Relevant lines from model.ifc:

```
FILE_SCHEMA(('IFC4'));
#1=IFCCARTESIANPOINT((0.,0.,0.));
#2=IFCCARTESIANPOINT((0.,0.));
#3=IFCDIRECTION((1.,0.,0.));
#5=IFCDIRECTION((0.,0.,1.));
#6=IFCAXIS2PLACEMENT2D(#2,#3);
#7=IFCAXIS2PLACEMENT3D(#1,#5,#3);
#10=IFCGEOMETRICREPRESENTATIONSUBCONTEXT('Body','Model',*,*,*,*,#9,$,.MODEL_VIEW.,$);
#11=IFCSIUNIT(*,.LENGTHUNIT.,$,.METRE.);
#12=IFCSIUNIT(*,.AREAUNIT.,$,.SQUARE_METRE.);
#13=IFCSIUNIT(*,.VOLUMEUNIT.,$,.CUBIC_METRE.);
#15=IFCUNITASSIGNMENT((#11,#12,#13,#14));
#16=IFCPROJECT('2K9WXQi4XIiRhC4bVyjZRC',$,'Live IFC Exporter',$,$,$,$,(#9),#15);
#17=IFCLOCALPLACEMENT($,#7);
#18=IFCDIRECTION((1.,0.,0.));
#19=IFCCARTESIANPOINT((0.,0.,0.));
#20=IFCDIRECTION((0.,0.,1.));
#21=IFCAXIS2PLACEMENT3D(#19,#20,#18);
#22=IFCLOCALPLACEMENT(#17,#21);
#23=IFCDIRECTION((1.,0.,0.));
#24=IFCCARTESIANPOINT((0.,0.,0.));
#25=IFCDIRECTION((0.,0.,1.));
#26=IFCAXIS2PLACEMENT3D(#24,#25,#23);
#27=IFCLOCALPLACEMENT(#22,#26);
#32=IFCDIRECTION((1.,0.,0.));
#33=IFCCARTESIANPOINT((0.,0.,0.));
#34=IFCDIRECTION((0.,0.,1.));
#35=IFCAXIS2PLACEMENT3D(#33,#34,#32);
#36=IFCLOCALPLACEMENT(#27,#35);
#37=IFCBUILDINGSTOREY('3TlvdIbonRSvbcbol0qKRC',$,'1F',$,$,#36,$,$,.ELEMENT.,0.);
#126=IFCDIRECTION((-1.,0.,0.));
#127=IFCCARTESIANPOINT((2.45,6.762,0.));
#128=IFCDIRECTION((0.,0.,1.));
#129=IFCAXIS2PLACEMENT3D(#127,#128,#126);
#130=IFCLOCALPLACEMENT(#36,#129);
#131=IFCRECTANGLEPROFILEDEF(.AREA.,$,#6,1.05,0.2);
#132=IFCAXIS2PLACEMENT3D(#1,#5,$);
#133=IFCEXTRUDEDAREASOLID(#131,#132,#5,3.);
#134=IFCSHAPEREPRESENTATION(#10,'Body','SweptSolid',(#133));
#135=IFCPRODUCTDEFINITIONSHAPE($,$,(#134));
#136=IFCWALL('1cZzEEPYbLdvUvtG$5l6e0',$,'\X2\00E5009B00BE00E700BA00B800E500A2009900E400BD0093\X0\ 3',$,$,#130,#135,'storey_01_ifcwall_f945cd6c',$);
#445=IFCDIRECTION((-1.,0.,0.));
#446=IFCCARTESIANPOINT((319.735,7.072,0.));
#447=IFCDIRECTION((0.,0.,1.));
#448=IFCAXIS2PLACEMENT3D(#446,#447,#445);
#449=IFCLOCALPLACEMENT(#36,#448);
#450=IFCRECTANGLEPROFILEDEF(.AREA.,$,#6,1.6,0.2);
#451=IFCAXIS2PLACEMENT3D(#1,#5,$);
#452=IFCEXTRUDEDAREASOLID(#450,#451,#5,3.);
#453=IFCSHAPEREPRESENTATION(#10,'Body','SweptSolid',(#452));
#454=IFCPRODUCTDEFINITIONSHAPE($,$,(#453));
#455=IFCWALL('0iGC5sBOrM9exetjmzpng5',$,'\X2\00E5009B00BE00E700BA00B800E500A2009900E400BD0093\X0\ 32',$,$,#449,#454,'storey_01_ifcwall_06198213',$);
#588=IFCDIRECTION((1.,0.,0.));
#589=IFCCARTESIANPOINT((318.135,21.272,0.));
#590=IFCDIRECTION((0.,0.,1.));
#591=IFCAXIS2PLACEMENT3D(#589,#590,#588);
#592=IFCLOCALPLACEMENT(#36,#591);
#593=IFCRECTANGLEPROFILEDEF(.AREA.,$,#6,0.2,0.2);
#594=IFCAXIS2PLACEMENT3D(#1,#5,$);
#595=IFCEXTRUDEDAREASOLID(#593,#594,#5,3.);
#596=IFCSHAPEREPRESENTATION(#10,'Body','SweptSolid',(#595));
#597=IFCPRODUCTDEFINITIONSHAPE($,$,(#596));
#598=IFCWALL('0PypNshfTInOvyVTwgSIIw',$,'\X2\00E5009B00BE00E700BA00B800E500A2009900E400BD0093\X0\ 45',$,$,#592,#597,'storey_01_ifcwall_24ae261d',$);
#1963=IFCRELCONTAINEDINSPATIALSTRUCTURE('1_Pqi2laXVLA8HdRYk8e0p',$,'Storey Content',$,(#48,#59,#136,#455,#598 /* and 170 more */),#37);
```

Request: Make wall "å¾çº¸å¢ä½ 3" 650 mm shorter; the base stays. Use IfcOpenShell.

```python
import ifcopenshell
import ifcopenshell.geom
import ifcopenshell.util.representation
import ifcopenshell.util.shape
import ifcopenshell.util.unit

model = ifcopenshell.open("model.ifc")
unit_scale = ifcopenshell.util.unit.calculate_unit_scale(model)
settings = ifcopenshell.geom.settings()


def volume(element):
    """Net volume in cubic metres, openings subtracted."""
    shape = ifcopenshell.geom.create_shape(settings, element)
    return ifcopenshell.util.shape.get_volume(shape.geometry)


wall = model.by_id(136)
before = volume(wall)

body = ifcopenshell.util.representation.get_representation(wall, "Model", "Body")
solid = body.Items[0]
old_height = solid.Depth
solid.Depth -= 0.65 / unit_scale
after = volume(wall)

print(f"height {old_height:g} -> {solid.Depth:g}, volume {before:.3f} -> {after:.3f} m3")

model.write("model_rev.ifc")
```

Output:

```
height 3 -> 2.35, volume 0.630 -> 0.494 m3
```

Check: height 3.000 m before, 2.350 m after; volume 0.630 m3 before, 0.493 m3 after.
